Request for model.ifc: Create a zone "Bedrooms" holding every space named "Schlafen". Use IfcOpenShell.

First a look at what the model holds.

```python
import ifcopenshell

model = ifcopenshell.open("model.ifc")
print(model.schema)
seen = {}
for space in model.by_type("IfcSpace"):
    seen[space.LongName] = seen.get(space.LongName, 0) + 1
for name, count in sorted(seen.items(), key=str):
    print(count, "x", name)
print("zones:", [z.Name for z in model.by_type("IfcZone")][:20])
```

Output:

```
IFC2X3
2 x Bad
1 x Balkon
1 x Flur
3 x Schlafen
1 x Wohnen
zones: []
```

```python
import ifcopenshell
import ifcopenshell.api.group
import ifcopenshell.api.root

model = ifcopenshell.open("model.ifc")

names = {"Schlafen"}
spaces = [s for s in model.by_type("IfcSpace") if s.LongName in names]

zone = ifcopenshell.api.root.create_entity(model, ifc_class="IfcZone", name="Bedrooms")
ifcopenshell.api.group.assign_group(model, products=spaces, group=zone)
print(len(spaces), "spaces in", zone.Name)

model.write("model_edited.ifc")
```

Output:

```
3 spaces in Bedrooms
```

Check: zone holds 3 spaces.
